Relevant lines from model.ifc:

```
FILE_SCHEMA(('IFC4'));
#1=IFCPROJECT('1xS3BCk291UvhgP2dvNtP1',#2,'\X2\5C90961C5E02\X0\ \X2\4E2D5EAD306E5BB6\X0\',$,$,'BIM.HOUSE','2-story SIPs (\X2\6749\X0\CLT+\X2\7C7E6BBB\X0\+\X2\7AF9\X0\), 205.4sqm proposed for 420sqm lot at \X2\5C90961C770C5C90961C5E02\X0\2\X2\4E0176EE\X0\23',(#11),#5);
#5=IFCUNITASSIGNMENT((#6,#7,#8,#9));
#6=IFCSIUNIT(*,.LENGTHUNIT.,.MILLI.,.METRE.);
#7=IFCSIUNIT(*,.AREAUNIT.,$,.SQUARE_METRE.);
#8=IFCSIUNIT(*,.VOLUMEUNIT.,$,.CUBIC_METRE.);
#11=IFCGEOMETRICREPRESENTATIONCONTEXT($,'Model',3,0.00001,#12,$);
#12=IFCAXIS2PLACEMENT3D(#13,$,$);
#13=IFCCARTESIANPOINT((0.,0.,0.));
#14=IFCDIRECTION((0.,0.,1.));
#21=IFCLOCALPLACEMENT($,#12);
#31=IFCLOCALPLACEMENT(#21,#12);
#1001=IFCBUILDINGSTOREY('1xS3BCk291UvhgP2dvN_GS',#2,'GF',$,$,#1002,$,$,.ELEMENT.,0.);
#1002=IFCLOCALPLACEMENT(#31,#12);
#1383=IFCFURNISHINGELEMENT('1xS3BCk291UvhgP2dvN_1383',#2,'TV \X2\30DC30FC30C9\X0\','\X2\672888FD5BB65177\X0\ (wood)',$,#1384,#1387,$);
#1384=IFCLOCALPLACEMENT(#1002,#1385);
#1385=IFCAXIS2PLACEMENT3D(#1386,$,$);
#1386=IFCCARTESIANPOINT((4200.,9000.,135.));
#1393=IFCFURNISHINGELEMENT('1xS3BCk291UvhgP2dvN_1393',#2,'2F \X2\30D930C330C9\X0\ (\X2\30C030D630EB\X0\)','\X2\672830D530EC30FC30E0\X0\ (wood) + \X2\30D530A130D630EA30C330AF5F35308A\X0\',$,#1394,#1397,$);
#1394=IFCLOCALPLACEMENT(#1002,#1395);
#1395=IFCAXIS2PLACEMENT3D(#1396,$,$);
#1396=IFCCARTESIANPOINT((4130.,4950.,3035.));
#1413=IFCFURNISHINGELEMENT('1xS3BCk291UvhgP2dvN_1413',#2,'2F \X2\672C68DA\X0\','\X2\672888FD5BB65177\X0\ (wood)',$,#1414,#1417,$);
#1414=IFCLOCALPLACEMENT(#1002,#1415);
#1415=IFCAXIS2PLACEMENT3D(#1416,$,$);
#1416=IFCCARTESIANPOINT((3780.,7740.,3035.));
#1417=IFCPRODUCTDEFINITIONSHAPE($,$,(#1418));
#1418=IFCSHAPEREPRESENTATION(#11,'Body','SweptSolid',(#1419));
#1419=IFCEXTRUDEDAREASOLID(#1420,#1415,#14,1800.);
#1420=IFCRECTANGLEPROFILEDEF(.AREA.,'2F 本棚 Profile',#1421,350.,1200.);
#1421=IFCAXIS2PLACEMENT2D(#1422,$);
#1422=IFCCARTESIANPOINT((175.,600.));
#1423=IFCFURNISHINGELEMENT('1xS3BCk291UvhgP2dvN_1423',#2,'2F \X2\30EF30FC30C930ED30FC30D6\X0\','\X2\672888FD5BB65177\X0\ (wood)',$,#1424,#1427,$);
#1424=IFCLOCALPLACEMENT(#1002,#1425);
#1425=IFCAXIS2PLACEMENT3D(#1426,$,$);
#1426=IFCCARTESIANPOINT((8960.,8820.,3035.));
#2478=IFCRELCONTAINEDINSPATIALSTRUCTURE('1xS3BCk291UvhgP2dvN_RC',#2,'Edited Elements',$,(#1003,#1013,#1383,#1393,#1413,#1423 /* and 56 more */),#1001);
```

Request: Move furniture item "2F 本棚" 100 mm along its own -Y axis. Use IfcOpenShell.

```python
import ifcopenshell
import ifcopenshell.api.geometry
import ifcopenshell.util.placement
import ifcopenshell.util.unit

model = ifcopenshell.open("model.ifc")
unit_scale = ifcopenshell.util.unit.calculate_unit_scale(model)

item = model.by_id(1413)
matrix = ifcopenshell.util.placement.get_local_placement(item.ObjectPlacement)
matrix[:3, 3] -= matrix[:3, 1] * 0.1 / unit_scale
ifcopenshell.api.geometry.edit_object_placement(model, product=item, matrix=matrix, is_si=False)

print(ifcopenshell.util.placement.get_local_placement(item.ObjectPlacement).round(3) + 0.0)

model.write("model_rev.ifc")
```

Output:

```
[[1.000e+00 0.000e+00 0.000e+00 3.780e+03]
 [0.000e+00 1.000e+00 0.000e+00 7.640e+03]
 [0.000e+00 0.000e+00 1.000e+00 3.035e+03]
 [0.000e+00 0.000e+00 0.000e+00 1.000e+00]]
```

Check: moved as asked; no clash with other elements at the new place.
